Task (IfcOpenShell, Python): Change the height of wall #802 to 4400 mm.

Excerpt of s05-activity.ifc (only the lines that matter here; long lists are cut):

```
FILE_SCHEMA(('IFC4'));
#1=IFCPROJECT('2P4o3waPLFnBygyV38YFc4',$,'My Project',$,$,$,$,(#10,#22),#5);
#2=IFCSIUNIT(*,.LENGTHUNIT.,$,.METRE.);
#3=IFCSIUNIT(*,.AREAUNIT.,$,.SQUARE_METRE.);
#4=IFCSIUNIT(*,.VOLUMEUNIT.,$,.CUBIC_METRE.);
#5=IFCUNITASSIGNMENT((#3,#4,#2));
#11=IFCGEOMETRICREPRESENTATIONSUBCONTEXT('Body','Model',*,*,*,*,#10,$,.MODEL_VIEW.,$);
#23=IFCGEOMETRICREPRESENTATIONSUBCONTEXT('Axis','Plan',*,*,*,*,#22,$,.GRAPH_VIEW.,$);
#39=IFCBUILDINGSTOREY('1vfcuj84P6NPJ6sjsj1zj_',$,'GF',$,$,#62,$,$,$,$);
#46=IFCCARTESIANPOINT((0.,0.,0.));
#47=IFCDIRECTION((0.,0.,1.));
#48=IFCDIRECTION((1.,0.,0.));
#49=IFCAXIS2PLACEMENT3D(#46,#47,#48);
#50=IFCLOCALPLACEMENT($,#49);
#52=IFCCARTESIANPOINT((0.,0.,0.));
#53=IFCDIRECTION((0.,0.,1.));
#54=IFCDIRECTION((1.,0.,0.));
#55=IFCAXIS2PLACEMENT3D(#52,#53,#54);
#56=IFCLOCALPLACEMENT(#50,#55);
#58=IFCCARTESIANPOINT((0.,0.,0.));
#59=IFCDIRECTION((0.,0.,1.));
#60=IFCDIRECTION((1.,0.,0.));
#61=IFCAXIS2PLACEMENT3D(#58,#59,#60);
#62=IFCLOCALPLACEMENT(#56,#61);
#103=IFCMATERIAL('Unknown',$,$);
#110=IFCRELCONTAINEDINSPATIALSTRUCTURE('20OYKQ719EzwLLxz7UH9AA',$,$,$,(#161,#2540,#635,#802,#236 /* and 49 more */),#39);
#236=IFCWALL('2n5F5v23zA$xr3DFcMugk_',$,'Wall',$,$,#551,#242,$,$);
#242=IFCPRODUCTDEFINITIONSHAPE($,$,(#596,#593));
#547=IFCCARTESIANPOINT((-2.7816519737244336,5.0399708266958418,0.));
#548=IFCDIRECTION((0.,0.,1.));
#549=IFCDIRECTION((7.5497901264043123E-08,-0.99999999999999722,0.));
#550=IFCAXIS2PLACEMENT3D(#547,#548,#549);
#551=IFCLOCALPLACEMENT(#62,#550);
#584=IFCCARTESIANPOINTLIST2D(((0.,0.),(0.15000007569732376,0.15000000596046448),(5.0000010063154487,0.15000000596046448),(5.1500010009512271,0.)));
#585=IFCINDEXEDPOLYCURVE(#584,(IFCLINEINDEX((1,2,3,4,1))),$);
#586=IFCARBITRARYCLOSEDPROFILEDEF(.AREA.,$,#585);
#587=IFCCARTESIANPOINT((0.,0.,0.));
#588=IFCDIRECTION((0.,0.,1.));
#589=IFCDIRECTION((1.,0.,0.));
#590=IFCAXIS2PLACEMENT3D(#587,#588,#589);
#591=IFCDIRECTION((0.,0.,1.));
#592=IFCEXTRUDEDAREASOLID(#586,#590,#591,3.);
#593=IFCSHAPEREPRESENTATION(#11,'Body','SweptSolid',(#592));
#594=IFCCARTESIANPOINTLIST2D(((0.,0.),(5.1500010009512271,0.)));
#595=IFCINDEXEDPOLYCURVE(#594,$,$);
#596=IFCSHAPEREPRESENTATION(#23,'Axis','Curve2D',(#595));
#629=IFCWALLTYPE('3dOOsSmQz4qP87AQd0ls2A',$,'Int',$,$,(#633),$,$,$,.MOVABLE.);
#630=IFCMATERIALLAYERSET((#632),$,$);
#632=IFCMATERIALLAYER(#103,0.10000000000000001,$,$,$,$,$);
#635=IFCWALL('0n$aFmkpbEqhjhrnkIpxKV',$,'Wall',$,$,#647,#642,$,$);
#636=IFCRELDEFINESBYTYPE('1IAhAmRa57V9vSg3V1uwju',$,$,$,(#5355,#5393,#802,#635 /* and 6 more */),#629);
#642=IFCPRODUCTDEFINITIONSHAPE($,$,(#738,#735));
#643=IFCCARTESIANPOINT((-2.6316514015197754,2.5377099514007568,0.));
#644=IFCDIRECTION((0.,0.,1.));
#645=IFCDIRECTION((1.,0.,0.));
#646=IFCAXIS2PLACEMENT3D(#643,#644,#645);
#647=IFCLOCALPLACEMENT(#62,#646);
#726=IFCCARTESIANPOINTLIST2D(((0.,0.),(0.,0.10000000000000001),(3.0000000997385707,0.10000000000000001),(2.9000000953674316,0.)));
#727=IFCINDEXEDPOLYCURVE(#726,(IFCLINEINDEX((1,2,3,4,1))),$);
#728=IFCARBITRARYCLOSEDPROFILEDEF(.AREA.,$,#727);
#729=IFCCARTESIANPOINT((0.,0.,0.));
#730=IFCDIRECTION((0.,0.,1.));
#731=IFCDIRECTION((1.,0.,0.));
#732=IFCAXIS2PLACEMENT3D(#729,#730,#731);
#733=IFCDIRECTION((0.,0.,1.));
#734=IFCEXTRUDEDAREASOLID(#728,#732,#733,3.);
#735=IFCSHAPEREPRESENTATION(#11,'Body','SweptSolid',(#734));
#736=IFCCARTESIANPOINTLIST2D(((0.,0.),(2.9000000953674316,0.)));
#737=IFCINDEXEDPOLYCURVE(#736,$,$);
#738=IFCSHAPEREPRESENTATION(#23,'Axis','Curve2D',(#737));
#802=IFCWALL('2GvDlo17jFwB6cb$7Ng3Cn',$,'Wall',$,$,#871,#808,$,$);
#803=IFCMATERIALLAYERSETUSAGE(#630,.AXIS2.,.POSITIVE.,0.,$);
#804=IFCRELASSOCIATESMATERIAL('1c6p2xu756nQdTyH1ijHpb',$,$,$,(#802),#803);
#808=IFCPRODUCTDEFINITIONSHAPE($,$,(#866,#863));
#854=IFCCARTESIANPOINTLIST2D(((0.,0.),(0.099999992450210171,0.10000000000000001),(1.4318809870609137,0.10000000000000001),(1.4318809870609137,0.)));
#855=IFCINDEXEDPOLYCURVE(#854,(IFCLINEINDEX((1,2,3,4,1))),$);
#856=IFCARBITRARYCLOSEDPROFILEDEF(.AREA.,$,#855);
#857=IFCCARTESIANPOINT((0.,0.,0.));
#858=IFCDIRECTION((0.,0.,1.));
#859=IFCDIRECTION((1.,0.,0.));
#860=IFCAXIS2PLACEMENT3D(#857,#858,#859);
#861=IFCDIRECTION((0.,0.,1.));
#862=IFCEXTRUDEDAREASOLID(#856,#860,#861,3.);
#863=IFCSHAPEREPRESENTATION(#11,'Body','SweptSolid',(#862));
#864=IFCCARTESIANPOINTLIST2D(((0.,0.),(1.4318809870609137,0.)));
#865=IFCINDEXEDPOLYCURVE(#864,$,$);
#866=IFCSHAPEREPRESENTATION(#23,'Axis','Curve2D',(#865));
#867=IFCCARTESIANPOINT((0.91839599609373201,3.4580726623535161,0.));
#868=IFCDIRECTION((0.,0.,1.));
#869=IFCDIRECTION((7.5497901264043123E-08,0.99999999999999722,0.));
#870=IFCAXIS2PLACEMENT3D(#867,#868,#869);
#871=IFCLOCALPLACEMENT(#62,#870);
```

```python
import ifcopenshell
import ifcopenshell.geom
import ifcopenshell.util.representation
import ifcopenshell.util.shape

model = ifcopenshell.open("s05-activity.ifc")
settings = ifcopenshell.geom.settings()


def volume(element):
    """Net volume in cubic metres, openings subtracted."""
    shape = ifcopenshell.geom.create_shape(settings, element)
    return ifcopenshell.util.shape.get_volume(shape.geometry)


wall = model.by_id(802)
before = volume(wall)

body = ifcopenshell.util.representation.get_representation(wall, "Model", "Body")
solid = body.Items[0]
old_height = solid.Depth
solid.Depth = 4.4
after = volume(wall)

print(f"height {old_height:g} -> {solid.Depth:g}, volume {before:.3f} -> {after:.3f} m3")

model.write("s05-activity_updated.ifc")
```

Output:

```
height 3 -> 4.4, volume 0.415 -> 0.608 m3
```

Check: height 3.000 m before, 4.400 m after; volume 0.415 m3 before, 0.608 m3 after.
